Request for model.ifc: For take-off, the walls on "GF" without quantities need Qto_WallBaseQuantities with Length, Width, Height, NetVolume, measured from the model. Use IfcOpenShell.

First a look at what the model holds.

```python
import ifcopenshell
import ifcopenshell.util.element
import ifcopenshell.util.unit

model = ifcopenshell.open("model.ifc")
print(model.schema)
for unit_type in ("LENGTHUNIT", "AREAUNIT", "VOLUMEUNIT"):
    print(unit_type, ifcopenshell.util.unit.calculate_unit_scale(model, unit_type))
storey = next(s for s in model.by_type("IfcBuildingStorey") if s.Name == "GF")
walls = [e for e in ifcopenshell.util.element.get_decomposition(storey) if e.is_a("IfcWall")]
for e in sorted(walls, key=lambda e: e.id()):
    print(e.id(), e.is_a(), e.Name, list(ifcopenshell.util.element.get_psets(e, qtos_only=True)), sep=" | ")
```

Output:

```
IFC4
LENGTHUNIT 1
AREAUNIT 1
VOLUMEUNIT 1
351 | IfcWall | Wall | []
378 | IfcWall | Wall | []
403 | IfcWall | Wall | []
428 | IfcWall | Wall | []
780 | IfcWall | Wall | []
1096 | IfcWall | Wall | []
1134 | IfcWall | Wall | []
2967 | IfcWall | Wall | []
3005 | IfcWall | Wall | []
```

```python
import ifcopenshell
import ifcopenshell.api.pset
import ifcopenshell.geom
import ifcopenshell.util.element
import ifcopenshell.util.shape
import ifcopenshell.util.unit

model = ifcopenshell.open("model.ifc")
unit_scale = ifcopenshell.util.unit.calculate_unit_scale(model)
volume_scale = ifcopenshell.util.unit.calculate_unit_scale(model, "VOLUMEUNIT")
settings = ifcopenshell.geom.settings()

storey = next(s for s in model.by_type("IfcBuildingStorey") if s.Name == "GF")
walls = [e for e in ifcopenshell.util.element.get_decomposition(storey) if e.is_a("IfcWall")]

for e in sorted(walls, key=lambda e: e.id()):
    if ifcopenshell.util.element.get_psets(e, qtos_only=True, should_inherit=False):
        continue
    # Geometry comes back in metres, in the element's own axes.
    shape = ifcopenshell.geom.create_shape(settings, e)
    values = {
        "Length": ifcopenshell.util.shape.get_x(shape.geometry) / unit_scale,
        "Width": ifcopenshell.util.shape.get_y(shape.geometry) / unit_scale,
        "Height": ifcopenshell.util.shape.get_z(shape.geometry) / unit_scale,
        "NetVolume": ifcopenshell.util.shape.get_volume(shape.geometry) / volume_scale,
    }
    qto = ifcopenshell.api.pset.add_qto(model, product=e, name="Qto_WallBaseQuantities")
    ifcopenshell.api.pset.edit_qto(model, qto=qto, properties=values)
    print(e.id(), {k: round(v, 3) for k, v in values.items()})

model.write("model_v2.ifc")
```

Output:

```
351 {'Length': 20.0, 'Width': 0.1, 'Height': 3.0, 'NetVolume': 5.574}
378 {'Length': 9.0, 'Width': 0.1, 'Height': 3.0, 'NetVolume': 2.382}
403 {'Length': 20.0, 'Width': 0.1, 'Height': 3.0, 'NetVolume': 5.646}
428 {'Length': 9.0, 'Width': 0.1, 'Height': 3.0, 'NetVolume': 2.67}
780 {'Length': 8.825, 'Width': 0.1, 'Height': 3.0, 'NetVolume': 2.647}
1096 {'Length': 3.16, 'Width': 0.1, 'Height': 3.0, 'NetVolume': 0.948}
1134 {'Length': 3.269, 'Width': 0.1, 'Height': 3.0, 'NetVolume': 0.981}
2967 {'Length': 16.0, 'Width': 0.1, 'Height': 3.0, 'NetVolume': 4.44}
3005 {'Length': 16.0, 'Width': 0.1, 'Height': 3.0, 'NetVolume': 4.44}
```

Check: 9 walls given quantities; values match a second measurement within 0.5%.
